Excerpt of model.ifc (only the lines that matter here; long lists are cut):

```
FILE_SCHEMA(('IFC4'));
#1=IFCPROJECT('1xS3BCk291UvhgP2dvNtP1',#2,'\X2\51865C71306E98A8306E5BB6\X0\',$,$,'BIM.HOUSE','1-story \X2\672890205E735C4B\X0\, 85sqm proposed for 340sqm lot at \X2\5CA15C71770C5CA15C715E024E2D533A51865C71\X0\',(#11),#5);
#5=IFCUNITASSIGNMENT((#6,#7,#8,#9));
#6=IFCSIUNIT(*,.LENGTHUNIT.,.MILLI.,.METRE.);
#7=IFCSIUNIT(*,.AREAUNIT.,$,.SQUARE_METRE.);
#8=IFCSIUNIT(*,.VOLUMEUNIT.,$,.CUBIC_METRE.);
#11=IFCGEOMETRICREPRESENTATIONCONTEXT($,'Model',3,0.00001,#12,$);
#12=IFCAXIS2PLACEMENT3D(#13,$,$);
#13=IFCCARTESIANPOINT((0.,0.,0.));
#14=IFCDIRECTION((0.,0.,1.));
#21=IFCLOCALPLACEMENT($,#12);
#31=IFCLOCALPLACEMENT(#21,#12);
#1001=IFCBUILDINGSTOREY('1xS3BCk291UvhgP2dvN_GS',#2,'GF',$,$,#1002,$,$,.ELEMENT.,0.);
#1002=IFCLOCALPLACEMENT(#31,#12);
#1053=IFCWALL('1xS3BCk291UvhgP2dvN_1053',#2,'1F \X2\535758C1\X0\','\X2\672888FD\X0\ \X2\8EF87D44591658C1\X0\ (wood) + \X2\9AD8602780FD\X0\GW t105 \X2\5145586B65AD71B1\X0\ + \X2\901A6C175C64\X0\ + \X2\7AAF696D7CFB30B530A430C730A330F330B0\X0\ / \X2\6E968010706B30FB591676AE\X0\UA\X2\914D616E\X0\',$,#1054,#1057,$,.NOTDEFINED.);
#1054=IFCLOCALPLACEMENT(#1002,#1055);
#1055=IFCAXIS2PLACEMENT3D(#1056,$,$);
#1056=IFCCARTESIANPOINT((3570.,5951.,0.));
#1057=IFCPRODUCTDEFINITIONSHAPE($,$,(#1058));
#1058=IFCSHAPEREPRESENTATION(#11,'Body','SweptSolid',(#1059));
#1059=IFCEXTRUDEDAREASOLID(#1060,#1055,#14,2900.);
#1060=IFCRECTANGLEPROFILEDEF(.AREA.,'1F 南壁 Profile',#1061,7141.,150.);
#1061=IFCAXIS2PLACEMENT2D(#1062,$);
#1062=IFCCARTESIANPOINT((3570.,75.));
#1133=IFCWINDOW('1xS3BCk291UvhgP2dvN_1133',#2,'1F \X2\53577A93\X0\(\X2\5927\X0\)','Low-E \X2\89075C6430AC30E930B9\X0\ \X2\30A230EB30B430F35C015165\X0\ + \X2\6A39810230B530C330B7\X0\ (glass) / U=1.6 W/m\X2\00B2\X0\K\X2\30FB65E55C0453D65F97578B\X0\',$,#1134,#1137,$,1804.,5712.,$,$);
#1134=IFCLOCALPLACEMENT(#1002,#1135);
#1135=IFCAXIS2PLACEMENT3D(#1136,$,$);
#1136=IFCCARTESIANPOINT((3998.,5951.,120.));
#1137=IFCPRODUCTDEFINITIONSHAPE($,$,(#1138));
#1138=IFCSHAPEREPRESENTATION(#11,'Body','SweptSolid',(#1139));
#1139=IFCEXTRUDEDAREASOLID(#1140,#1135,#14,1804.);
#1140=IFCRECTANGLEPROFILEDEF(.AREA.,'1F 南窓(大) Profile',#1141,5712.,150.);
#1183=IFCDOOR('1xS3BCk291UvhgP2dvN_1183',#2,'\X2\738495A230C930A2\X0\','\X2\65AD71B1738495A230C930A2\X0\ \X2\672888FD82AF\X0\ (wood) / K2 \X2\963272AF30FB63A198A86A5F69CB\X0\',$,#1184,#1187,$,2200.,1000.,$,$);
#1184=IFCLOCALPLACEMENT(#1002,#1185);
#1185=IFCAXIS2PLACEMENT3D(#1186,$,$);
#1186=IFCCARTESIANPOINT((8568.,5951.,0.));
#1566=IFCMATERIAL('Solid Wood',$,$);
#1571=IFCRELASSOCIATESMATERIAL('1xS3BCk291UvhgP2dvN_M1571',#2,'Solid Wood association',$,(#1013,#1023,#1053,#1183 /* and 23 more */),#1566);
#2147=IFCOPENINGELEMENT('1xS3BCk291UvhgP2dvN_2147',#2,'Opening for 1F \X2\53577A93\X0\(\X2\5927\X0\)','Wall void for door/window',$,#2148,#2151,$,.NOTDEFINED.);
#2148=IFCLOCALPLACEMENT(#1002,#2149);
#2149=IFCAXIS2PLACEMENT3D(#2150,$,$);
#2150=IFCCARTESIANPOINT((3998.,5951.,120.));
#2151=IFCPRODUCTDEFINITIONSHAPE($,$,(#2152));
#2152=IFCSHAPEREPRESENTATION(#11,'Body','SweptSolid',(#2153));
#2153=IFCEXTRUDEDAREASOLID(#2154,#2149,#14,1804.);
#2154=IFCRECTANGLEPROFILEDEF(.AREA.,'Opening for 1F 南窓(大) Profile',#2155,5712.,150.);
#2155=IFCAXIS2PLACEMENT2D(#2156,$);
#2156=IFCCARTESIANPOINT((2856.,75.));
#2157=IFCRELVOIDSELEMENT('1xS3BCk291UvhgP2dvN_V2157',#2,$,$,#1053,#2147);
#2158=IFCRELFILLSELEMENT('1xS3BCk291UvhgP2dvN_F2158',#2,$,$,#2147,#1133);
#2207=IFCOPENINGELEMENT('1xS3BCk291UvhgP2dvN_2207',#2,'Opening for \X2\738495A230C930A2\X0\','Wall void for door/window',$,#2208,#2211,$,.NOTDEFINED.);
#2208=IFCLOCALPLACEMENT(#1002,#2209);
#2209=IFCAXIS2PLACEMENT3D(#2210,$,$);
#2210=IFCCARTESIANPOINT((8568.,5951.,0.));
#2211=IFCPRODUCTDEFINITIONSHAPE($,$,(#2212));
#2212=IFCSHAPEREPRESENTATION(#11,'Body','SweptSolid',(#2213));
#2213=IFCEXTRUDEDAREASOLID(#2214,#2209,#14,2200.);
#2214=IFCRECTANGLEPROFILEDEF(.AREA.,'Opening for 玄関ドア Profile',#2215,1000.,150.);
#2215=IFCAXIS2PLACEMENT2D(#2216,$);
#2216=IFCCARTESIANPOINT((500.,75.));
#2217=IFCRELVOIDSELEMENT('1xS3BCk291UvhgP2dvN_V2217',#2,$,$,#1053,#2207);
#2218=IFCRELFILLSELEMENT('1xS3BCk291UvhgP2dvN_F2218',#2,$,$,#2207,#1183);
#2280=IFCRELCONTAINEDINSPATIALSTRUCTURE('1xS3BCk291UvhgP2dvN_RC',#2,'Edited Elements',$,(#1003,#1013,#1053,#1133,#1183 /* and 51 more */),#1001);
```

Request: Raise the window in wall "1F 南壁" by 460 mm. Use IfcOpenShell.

```python
import numpy as np
import ifcopenshell
import ifcopenshell.api.geometry
import ifcopenshell.util.placement
import ifcopenshell.util.unit

model = ifcopenshell.open("model.ifc")
unit_scale = ifcopenshell.util.unit.calculate_unit_scale(model)

window = model.by_id(1133)
opening = window.FillsVoids[0].RelatingOpeningElement
dz = 0.46 / unit_scale

shift = np.array([0.0, 0.0, dz])
# The window is not placed relative to its opening, so move both.
for product in (opening, window):
    matrix = ifcopenshell.util.placement.get_local_placement(product.ObjectPlacement)
    matrix[:3, 3] += shift
    ifcopenshell.api.geometry.edit_object_placement(model, product=product, matrix=matrix, is_si=False)

print(f"moved by {dz * unit_scale:+.3f} m")

model.write("model-out.ifc")
```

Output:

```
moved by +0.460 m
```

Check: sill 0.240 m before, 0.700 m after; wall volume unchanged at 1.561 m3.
